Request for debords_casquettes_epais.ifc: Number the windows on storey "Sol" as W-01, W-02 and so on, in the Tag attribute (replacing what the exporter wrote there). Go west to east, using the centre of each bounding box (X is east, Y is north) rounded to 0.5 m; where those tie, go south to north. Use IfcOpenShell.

First a look at what the model holds.

```python
import ifcopenshell
import ifcopenshell.util.element
import ifcopenshell.util.placement

model = ifcopenshell.open("debords_casquettes_epais.ifc")
print(model.schema)
storey = next(s for s in model.by_type("IfcBuildingStorey") if s.Name == "Sol")
windows = [e for e in ifcopenshell.util.element.get_decomposition(storey) if e.is_a("IfcWindow")]
for e in sorted(windows, key=lambda e: e.id()):
    origin = ifcopenshell.util.placement.get_local_placement(e.ObjectPlacement)[:3, 3]
    print(e.id(), e.Tag, e.Name, origin.round(2) + 0.0, sep=" | ")
```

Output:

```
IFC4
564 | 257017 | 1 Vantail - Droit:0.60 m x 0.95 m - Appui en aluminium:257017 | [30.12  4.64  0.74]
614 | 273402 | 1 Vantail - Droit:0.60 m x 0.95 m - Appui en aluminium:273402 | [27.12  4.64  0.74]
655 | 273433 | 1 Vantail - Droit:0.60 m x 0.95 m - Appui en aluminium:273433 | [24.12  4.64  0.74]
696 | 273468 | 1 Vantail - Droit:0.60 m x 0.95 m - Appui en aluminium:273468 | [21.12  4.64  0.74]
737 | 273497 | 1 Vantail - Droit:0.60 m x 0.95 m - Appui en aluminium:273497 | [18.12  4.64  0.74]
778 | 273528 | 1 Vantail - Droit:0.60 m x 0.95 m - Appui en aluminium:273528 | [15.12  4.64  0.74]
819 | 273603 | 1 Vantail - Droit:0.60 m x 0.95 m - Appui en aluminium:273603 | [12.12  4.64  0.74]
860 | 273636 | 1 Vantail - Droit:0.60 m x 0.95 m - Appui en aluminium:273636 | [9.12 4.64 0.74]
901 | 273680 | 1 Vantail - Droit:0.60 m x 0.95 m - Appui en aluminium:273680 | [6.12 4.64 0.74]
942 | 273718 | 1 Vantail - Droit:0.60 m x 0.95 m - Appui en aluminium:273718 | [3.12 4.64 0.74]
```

```python
import ifcopenshell
import ifcopenshell.geom
import ifcopenshell.util.element
import ifcopenshell.util.shape

model = ifcopenshell.open("debords_casquettes_epais.ifc")
settings = ifcopenshell.geom.settings()
settings.set("use-world-coords", True)


def centre(element):
    shape = ifcopenshell.geom.create_shape(settings, element)
    return ifcopenshell.util.shape.get_bbox_centroid(shape.geometry)


storey = next(s for s in model.by_type("IfcBuildingStorey") if s.Name == "Sol")
windows = [e for e in ifcopenshell.util.element.get_decomposition(storey) if e.is_a("IfcWindow")]

# Insertion points can sit at a corner or the storey origin, so sort by the geometry (in metres).
centres = {e: centre(e) for e in windows}
windows.sort(key=lambda e: (round(centres[e][0] / 0.5), centres[e][1]))

for i, e in enumerate(windows, start=1):
    number = f"W-{i:02d}"
    e.Tag = number
    print(e.id(), number)

model.write("debords_casquettes_epais_rev.ifc")
```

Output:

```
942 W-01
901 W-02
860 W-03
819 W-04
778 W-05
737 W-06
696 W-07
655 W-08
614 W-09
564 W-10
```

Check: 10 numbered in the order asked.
